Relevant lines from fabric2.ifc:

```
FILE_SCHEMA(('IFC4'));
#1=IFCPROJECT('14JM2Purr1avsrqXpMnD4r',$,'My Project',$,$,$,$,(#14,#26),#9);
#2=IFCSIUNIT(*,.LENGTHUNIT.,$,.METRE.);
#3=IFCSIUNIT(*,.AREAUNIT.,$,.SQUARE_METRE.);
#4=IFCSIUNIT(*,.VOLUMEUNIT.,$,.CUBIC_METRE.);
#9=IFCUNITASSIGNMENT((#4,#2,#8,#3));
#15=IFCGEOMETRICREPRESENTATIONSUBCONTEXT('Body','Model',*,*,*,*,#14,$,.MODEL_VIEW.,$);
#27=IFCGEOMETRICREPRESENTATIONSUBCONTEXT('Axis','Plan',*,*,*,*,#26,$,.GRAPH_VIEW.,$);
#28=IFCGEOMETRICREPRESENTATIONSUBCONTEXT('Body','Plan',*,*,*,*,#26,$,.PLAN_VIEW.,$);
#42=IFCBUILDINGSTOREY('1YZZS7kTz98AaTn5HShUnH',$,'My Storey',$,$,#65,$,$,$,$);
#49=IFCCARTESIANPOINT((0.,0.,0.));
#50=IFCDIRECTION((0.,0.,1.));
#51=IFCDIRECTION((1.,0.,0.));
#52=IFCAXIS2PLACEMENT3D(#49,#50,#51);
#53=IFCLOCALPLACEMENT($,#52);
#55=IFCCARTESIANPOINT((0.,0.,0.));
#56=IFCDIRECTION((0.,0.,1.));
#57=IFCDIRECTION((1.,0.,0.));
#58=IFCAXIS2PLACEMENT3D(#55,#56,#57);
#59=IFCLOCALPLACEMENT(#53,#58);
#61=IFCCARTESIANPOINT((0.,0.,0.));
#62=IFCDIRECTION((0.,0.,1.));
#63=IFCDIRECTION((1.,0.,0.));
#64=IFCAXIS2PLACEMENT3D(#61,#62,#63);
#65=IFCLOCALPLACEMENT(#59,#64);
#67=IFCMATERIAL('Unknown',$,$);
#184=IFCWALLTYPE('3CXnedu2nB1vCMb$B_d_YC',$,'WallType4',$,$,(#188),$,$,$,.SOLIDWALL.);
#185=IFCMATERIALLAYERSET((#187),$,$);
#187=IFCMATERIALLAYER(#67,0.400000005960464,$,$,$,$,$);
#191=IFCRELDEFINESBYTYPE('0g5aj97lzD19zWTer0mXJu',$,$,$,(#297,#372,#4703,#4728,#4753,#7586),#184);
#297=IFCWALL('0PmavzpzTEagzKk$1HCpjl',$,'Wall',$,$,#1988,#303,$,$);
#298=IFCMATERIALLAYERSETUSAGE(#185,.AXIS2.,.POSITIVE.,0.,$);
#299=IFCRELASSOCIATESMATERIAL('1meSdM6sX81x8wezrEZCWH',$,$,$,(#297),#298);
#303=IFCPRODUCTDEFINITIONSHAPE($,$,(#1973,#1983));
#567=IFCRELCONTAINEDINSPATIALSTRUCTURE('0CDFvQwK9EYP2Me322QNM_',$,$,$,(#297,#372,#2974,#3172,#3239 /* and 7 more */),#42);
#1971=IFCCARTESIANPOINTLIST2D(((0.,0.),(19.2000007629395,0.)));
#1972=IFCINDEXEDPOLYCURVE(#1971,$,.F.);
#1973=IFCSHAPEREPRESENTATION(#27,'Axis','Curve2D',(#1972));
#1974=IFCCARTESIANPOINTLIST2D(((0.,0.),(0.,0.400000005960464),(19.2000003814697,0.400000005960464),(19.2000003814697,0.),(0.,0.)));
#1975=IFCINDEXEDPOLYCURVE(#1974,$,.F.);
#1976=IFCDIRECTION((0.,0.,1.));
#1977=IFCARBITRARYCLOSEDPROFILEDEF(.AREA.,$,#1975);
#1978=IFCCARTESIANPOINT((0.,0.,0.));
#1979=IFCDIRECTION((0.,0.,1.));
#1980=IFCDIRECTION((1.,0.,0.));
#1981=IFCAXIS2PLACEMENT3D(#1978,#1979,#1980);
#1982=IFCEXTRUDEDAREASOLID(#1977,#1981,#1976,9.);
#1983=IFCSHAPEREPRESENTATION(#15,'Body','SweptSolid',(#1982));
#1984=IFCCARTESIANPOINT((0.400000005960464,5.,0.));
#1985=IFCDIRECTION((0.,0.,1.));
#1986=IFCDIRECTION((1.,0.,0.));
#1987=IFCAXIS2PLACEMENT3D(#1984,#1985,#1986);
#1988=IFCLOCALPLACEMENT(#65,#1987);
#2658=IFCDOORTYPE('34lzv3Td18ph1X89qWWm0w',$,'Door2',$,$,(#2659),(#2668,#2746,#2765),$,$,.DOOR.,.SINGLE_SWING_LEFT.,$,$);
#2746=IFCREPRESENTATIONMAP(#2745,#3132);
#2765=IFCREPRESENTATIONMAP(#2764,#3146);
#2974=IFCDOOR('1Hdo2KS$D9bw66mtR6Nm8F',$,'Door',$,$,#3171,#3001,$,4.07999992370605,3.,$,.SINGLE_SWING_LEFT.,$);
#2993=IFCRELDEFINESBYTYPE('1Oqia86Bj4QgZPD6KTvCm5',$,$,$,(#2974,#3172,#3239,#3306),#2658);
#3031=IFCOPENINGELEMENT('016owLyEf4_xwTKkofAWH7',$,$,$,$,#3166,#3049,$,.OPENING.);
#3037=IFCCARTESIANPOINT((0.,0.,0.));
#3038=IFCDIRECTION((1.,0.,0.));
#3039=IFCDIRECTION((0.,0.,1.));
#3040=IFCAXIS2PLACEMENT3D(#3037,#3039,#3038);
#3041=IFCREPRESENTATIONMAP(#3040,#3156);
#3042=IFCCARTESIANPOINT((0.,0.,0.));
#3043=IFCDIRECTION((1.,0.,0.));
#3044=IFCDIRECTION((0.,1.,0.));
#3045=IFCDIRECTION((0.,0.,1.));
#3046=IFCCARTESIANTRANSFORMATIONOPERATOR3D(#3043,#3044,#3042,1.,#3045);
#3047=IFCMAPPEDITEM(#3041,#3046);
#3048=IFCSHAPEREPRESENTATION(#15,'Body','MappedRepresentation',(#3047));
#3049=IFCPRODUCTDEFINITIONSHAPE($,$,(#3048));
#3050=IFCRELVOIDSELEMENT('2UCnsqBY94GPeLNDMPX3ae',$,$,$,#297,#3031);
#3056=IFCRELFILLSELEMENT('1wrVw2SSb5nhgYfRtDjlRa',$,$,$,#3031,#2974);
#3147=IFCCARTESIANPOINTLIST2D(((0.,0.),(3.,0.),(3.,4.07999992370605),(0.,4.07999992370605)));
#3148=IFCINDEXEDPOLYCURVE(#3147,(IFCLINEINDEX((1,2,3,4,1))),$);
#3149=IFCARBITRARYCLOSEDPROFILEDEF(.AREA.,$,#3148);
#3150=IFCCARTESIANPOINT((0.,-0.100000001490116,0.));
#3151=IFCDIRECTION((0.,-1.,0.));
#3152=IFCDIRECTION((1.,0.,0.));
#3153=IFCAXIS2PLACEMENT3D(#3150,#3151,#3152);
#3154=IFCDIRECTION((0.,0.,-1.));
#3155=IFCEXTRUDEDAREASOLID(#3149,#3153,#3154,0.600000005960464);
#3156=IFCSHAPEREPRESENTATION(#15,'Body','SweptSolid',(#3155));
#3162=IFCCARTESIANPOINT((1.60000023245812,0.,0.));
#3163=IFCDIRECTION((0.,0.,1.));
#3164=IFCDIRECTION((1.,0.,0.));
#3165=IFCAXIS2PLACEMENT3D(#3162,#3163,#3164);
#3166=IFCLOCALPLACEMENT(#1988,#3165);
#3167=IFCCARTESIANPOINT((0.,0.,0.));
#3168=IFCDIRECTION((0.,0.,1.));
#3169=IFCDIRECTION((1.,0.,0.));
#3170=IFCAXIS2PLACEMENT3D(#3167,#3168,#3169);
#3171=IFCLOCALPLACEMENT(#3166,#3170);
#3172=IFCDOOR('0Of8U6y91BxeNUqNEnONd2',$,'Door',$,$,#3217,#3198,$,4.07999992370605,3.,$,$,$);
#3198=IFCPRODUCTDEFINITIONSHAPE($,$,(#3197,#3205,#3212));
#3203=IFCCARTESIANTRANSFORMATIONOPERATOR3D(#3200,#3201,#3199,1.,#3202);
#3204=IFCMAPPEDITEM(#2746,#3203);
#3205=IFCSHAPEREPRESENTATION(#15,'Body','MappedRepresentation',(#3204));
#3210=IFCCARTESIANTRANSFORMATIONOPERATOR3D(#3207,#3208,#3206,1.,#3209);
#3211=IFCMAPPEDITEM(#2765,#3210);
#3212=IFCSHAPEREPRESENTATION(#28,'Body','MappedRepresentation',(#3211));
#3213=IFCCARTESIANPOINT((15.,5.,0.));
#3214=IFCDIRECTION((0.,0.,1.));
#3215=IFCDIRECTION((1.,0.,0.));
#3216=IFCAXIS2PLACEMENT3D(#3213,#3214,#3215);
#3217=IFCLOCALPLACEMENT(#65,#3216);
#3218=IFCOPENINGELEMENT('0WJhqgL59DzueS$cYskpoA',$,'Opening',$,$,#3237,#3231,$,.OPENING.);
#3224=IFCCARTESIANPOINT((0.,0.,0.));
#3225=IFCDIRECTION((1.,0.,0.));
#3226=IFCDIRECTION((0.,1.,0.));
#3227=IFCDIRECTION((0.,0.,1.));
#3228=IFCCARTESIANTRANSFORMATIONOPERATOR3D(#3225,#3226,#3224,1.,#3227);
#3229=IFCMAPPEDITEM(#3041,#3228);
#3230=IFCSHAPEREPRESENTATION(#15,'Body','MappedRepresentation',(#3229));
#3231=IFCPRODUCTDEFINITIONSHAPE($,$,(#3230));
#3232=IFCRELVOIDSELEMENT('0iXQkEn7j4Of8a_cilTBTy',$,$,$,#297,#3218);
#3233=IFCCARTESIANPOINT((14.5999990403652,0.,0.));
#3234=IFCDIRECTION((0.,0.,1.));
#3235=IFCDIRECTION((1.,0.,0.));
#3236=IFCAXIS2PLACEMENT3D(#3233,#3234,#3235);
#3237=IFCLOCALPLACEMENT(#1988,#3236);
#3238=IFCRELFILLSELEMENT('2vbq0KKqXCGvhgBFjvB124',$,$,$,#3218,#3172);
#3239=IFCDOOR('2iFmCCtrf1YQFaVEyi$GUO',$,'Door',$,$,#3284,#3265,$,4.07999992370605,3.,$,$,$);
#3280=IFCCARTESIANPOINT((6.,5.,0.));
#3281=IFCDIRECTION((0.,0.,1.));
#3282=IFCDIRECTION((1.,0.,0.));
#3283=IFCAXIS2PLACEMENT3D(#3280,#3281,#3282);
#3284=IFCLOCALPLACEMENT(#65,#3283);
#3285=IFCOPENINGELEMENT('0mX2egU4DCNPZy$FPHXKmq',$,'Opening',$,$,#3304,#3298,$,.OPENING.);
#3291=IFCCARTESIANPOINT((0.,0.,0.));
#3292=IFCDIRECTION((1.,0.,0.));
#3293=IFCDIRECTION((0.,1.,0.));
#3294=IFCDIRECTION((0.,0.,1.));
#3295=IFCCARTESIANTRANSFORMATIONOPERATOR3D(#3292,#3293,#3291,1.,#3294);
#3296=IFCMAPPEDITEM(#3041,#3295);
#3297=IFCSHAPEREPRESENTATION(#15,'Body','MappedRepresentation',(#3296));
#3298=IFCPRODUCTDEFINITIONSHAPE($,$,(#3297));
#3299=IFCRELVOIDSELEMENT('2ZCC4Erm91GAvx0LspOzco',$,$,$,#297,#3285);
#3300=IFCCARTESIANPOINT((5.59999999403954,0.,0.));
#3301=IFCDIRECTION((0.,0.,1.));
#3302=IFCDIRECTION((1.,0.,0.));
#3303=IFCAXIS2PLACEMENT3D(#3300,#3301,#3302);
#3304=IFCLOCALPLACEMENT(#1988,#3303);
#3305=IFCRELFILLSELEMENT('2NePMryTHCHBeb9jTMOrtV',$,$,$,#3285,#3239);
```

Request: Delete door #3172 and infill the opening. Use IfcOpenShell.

```python
import ifcopenshell
import ifcopenshell.api.feature
import ifcopenshell.api.root
import ifcopenshell.geom
import ifcopenshell.util.shape

model = ifcopenshell.open("fabric2.ifc")
settings = ifcopenshell.geom.settings()


def volume(element):
    """Net volume in cubic metres, openings subtracted."""
    shape = ifcopenshell.geom.create_shape(settings, element)
    return ifcopenshell.util.shape.get_volume(shape.geometry)


door = model.by_guid("0Of8U6y91BxeNUqNEnONd2")
opening = door.FillsVoids[0].RelatingOpeningElement
wall = opening.VoidsElements[0].RelatingBuildingElement
before = volume(wall)

ifcopenshell.api.root.remove_product(model, product=door)
ifcopenshell.api.feature.remove_feature(model, feature=opening)

after = volume(wall)

print(f"wall volume {before:.3f} -> {after:.3f} m3")

model.write("fabric2-out.ifc")
```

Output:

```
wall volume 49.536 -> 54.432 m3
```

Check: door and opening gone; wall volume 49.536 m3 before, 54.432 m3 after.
